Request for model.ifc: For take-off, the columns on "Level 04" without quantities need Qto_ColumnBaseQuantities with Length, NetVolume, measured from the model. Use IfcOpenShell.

First a look at what the model holds.

```python
import ifcopenshell
import ifcopenshell.util.element
import ifcopenshell.util.unit

model = ifcopenshell.open("model.ifc")
print(model.schema)
for unit_type in ("LENGTHUNIT", "AREAUNIT", "VOLUMEUNIT"):
    print(unit_type, ifcopenshell.util.unit.calculate_unit_scale(model, unit_type))
storey = next(s for s in model.by_type("IfcBuildingStorey") if s.Name == "Level 04")
columns = [e for e in ifcopenshell.util.element.get_decomposition(storey) if e.is_a("IfcColumn")]
for e in sorted(columns, key=lambda e: e.id()):
    print(e.id(), e.is_a(), e.Name, list(ifcopenshell.util.element.get_psets(e, qtos_only=True)), sep=" | ")
```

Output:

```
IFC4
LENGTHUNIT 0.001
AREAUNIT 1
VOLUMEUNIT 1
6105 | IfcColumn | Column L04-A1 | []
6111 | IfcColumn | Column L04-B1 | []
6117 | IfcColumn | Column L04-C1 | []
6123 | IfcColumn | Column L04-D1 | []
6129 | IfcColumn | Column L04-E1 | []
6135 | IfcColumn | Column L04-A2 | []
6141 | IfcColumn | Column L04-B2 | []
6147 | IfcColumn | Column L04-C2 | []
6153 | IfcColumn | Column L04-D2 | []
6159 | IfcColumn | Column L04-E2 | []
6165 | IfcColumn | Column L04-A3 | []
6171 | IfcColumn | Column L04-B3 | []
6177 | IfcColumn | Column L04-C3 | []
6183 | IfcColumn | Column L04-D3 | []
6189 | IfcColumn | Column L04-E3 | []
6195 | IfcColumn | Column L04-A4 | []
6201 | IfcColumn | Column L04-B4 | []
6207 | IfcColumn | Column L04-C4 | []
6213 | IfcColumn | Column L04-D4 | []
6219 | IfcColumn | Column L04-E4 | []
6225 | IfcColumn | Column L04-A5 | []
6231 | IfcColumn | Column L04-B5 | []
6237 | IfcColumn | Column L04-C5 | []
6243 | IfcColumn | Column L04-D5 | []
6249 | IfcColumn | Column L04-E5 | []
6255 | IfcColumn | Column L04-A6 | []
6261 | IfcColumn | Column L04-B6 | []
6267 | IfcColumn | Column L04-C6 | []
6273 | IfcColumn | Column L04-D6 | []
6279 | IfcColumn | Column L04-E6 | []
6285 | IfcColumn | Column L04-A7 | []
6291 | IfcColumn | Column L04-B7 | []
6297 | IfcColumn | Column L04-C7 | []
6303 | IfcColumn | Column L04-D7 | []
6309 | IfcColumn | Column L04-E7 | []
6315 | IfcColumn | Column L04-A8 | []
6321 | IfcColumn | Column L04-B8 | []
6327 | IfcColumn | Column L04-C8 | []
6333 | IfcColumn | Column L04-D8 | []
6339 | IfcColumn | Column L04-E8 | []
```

```python
import ifcopenshell
import ifcopenshell.api.pset
import ifcopenshell.geom
import ifcopenshell.util.element
import ifcopenshell.util.shape
import ifcopenshell.util.unit

model = ifcopenshell.open("model.ifc")
unit_scale = ifcopenshell.util.unit.calculate_unit_scale(model)
volume_scale = ifcopenshell.util.unit.calculate_unit_scale(model, "VOLUMEUNIT")
settings = ifcopenshell.geom.settings()

storey = next(s for s in model.by_type("IfcBuildingStorey") if s.Name == "Level 04")
columns = [e for e in ifcopenshell.util.element.get_decomposition(storey) if e.is_a("IfcColumn")]

for e in sorted(columns, key=lambda e: e.id()):
    if ifcopenshell.util.element.get_psets(e, qtos_only=True, should_inherit=False):
        continue
    # Geometry comes back in metres, in the element's own axes.
    shape = ifcopenshell.geom.create_shape(settings, e)
    values = {
        "Length": ifcopenshell.util.shape.get_z(shape.geometry) / unit_scale,
        "NetVolume": ifcopenshell.util.shape.get_volume(shape.geometry) / volume_scale,
    }
    qto = ifcopenshell.api.pset.add_qto(model, product=e, name="Qto_ColumnBaseQuantities")
    ifcopenshell.api.pset.edit_qto(model, qto=qto, properties=values)
    print(e.id(), {k: round(v, 3) for k, v in values.items()})

model.write("model_rev.ifc")
```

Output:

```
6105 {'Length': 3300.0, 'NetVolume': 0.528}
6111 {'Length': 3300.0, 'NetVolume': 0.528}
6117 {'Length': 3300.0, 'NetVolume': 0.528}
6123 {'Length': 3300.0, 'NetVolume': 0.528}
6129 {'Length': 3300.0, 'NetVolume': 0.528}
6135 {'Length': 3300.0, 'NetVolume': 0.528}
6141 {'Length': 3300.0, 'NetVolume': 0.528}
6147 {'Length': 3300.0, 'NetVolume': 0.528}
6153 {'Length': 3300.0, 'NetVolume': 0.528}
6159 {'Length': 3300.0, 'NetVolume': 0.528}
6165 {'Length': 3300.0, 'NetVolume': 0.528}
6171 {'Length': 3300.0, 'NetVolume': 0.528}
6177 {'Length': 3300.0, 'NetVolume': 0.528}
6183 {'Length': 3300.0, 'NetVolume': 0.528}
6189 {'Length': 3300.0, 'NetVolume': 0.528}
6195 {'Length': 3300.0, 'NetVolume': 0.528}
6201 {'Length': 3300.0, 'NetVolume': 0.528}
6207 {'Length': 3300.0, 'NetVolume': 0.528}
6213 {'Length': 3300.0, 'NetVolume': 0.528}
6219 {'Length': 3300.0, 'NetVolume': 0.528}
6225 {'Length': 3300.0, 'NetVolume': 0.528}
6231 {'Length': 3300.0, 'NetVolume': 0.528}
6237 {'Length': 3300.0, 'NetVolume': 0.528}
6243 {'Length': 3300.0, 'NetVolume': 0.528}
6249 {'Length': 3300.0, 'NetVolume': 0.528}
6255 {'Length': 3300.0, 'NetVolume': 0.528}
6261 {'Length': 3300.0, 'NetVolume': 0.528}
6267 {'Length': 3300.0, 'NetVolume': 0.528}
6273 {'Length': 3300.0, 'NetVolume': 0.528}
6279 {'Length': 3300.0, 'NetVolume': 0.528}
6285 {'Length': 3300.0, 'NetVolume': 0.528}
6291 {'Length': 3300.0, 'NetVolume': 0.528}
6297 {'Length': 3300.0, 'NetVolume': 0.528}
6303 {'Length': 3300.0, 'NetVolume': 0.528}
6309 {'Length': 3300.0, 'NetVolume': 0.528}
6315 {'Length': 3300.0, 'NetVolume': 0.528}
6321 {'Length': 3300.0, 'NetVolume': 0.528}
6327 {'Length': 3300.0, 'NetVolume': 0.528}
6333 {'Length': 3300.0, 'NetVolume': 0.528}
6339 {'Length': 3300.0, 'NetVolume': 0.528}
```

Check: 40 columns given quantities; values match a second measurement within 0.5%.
